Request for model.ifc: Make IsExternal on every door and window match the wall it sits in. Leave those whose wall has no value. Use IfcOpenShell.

First a look at what the model holds.

```python
import ifcopenshell
import ifcopenshell.util.element

model = ifcopenshell.open("model.ifc")
print(model.schema)
seen = {}
for e in model.by_type("IfcDoor") + model.by_type("IfcWindow"):
    if not e.FillsVoids:
        continue
    host = e.FillsVoids[0].RelatingOpeningElement.VoidsElements[0].RelatingBuildingElement
    own = ifcopenshell.util.element.get_pset(e, f"Pset_{e.is_a()[3:].removesuffix('StandardCase')}Common", "IsExternal")
    wall = ifcopenshell.util.element.get_pset(host, "Pset_WallCommon", "IsExternal")
    seen[e.is_a(), own, wall] = seen.get((e.is_a(), own, wall), 0) + 1
for (cls, own, wall), count in sorted(seen.items(), key=str):
    print(count, cls, "IsExternal:", own, "| host wall:", wall)
```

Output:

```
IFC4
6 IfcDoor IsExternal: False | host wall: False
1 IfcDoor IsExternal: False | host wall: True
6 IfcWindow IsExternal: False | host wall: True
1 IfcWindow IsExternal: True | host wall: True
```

```python
import ifcopenshell
import ifcopenshell.api.pset
import ifcopenshell.util.element

model = ifcopenshell.open("model.ifc")

count = 0
for ifc_class, pset_name in (("IfcDoor", "Pset_DoorCommon"), ("IfcWindow", "Pset_WindowCommon")):
    for e in model.by_type(ifc_class):
        if not e.FillsVoids:
            continue
        host = e.FillsVoids[0].RelatingOpeningElement.VoidsElements[0].RelatingBuildingElement
        external = ifcopenshell.util.element.get_pset(host, "Pset_WallCommon", "IsExternal")
        if external is None or ifcopenshell.util.element.get_pset(e, pset_name, "IsExternal") == external:
            continue
        pset = ifcopenshell.api.pset.add_pset(model, product=e, name=pset_name)
        ifcopenshell.api.pset.edit_pset(model, pset=pset, properties={"IsExternal": external})
        count += 1

print(count, "updated")

model.write("model_edited.ifc")
```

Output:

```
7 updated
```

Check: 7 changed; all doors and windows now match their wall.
